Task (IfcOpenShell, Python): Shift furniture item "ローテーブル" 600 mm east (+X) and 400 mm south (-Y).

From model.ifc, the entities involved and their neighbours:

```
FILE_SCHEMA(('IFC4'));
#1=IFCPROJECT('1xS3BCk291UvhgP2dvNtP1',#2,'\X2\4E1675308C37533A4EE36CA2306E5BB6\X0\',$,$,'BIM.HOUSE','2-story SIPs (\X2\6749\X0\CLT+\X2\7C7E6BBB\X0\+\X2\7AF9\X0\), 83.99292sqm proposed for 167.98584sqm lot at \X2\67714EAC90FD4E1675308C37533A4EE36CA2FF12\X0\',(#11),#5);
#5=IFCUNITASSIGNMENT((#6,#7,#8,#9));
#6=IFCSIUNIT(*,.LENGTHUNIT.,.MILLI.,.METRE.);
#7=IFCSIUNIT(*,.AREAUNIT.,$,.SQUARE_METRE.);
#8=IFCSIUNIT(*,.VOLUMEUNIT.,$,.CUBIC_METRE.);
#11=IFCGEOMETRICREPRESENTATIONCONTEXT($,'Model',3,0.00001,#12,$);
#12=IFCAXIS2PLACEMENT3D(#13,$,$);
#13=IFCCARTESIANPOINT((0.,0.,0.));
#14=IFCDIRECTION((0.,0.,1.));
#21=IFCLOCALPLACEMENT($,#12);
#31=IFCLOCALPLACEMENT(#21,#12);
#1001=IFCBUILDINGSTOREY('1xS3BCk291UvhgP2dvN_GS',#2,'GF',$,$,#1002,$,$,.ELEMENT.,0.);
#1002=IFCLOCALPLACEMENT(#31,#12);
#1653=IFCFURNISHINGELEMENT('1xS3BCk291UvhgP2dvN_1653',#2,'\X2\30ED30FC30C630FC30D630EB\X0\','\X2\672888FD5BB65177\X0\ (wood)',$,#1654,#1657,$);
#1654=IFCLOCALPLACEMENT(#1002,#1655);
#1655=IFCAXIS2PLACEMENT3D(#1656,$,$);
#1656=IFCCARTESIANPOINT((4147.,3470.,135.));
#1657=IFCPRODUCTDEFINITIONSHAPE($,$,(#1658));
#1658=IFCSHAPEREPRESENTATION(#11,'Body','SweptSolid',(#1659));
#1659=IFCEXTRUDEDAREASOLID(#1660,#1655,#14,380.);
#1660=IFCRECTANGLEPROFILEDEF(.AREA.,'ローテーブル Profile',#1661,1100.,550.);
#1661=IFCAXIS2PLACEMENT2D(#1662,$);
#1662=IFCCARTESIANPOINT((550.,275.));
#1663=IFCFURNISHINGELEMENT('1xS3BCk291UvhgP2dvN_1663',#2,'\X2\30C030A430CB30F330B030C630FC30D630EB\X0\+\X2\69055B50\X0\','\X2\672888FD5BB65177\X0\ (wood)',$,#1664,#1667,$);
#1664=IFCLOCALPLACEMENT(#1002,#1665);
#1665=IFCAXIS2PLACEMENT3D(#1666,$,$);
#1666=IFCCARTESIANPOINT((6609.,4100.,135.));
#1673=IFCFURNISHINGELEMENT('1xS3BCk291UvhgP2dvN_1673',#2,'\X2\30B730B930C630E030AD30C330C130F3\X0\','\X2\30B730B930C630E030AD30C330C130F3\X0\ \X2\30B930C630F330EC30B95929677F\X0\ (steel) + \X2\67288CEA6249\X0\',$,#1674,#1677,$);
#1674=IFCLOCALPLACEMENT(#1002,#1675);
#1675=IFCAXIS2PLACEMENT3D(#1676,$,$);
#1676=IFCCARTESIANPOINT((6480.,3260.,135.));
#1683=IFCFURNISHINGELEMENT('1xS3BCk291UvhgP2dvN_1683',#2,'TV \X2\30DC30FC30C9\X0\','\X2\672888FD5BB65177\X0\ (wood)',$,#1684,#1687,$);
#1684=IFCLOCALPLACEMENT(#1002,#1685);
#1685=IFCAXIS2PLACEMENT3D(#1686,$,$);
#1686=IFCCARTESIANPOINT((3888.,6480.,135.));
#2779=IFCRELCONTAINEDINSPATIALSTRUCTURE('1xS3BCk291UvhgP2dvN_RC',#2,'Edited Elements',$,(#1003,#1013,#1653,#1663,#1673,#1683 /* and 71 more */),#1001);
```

```python
import ifcopenshell
import ifcopenshell.api.geometry
import ifcopenshell.util.placement

model = ifcopenshell.open("model.ifc")

item = model.by_id(1653)
matrix = ifcopenshell.util.placement.get_local_placement(item.ObjectPlacement)
matrix[0, 3] += 600.0
matrix[1, 3] -= 400.0
ifcopenshell.api.geometry.edit_object_placement(model, product=item, matrix=matrix, is_si=False)

print(ifcopenshell.util.placement.get_local_placement(item.ObjectPlacement).round(3) + 0.0)

model.write("model_updated.ifc")
```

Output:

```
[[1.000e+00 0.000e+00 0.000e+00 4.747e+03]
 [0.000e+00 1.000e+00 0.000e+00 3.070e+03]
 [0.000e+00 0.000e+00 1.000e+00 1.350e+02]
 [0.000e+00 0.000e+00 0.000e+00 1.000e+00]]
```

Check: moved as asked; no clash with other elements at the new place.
